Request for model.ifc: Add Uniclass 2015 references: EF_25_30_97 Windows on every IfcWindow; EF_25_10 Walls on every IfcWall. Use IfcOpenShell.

First a look at what the model holds.

```python
import ifcopenshell

model = ifcopenshell.open("model.ifc")
print(model.schema)
print("classifications:", [c.Name for c in model.by_type("IfcClassification")])
for ifc_class in ("IfcDoor", "IfcRoof", "IfcStair", "IfcWall", "IfcWindow"):
    print(ifc_class, len(model.by_type(ifc_class)))
```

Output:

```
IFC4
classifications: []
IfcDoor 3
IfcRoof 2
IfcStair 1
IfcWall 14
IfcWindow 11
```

```python
import ifcopenshell
import ifcopenshell.api.classification

model = ifcopenshell.open("model.ifc")

system = ifcopenshell.api.classification.add_classification(model, classification="Uniclass 2015")

codes = {
    "IfcWindow": ("EF_25_30_97", "Windows"),
    "IfcWall": ("EF_25_10", "Walls"),
}
for ifc_class, (code, name) in codes.items():
    products = model.by_type(ifc_class)
    ifcopenshell.api.classification.add_reference(
        model, products=products, classification=system, identification=code, name=name
    )
    print(code, len(products))

model.write("model_v2.ifc")
```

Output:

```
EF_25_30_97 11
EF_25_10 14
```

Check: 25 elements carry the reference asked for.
